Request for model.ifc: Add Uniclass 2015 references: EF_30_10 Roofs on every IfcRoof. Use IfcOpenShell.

First a look at what the model holds.

```python
import ifcopenshell

model = ifcopenshell.open("model.ifc")
print(model.schema)
print("classifications:", [c.Name for c in model.by_type("IfcClassification")])
for ifc_class in ("IfcDoor", "IfcRoof", "IfcStair", "IfcWall", "IfcWindow"):
    print(ifc_class, len(model.by_type(ifc_class)))
```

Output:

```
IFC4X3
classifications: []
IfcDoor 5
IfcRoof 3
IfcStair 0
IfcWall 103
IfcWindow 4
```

```python
import ifcopenshell
import ifcopenshell.api.classification

model = ifcopenshell.open("model.ifc")

system = ifcopenshell.api.classification.add_classification(model, classification="Uniclass 2015")

codes = {
    "IfcRoof": ("EF_30_10", "Roofs"),
}
for ifc_class, (code, name) in codes.items():
    products = model.by_type(ifc_class)
    ifcopenshell.api.classification.add_reference(
        model, products=products, classification=system, identification=code, name=name
    )
    print(code, len(products))

model.write("model-out.ifc")
```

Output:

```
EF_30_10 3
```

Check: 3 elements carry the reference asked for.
